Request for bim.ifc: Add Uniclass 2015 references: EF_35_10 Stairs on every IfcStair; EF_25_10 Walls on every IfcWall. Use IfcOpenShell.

First a look at what the model holds.

```python
import ifcopenshell

model = ifcopenshell.open("bim.ifc")
print(model.schema)
print("classifications:", [c.Name for c in model.by_type("IfcClassification")])
for ifc_class in ("IfcDoor", "IfcRoof", "IfcStair", "IfcWall", "IfcWindow"):
    print(ifc_class, len(model.by_type(ifc_class)))
```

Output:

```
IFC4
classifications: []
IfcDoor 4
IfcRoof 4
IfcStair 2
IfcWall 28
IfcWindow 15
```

```python
import ifcopenshell
import ifcopenshell.api.classification

model = ifcopenshell.open("bim.ifc")

system = ifcopenshell.api.classification.add_classification(model, classification="Uniclass 2015")

codes = {
    "IfcStair": ("EF_35_10", "Stairs"),
    "IfcWall": ("EF_25_10", "Walls"),
}
for ifc_class, (code, name) in codes.items():
    products = model.by_type(ifc_class)
    ifcopenshell.api.classification.add_reference(
        model, products=products, classification=system, identification=code, name=name
    )
    print(code, len(products))

model.write("bim_edited.ifc")
```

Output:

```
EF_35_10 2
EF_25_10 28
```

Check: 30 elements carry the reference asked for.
